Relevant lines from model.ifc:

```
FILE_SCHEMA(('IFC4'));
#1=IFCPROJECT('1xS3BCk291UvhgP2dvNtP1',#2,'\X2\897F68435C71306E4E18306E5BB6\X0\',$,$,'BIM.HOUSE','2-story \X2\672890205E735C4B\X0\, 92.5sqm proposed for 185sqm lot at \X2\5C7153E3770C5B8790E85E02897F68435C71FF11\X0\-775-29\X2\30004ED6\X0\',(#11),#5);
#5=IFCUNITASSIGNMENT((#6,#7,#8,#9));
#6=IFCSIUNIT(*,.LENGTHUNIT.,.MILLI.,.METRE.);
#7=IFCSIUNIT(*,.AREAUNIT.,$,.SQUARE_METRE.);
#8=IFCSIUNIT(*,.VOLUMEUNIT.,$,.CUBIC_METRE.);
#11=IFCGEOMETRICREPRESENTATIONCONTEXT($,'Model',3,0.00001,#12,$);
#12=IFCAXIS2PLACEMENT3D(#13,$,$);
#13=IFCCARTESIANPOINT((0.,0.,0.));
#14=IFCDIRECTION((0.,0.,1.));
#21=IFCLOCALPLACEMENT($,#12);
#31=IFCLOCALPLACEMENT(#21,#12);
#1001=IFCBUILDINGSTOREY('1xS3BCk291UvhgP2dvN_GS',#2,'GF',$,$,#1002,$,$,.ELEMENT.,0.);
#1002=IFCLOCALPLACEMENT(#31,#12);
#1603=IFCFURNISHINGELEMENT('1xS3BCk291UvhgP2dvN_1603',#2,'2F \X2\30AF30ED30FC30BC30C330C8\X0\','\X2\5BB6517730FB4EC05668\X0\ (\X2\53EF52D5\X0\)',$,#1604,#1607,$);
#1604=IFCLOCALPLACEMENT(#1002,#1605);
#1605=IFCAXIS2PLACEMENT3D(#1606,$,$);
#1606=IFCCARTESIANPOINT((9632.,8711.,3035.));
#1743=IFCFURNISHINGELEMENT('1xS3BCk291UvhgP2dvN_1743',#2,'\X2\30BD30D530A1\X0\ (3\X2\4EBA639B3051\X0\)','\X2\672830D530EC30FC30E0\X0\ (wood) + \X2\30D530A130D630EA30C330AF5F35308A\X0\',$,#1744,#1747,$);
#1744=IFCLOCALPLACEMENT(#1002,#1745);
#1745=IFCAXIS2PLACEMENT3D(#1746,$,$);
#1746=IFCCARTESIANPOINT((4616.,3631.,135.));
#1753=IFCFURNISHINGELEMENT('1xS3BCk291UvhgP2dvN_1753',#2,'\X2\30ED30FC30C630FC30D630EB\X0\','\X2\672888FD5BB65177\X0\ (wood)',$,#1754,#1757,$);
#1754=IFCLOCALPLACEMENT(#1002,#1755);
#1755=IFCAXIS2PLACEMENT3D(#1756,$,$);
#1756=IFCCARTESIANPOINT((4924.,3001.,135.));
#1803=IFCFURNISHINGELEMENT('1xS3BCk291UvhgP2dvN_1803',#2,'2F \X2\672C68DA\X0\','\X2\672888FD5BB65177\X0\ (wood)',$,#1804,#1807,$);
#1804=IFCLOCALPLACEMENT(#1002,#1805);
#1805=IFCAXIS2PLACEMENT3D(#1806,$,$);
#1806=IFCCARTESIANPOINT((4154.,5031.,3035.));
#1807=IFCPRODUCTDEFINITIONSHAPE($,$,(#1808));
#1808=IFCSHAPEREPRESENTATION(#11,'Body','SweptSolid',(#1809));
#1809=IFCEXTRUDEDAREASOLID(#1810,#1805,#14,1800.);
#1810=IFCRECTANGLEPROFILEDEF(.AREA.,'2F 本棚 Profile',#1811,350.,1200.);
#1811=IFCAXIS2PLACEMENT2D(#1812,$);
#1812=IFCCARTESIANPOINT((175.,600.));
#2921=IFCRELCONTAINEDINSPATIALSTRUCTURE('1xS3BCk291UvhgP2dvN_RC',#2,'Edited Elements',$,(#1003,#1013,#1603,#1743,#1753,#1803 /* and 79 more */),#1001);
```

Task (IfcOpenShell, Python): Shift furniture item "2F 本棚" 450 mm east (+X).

```python
import ifcopenshell
import ifcopenshell.api.geometry
import ifcopenshell.util.placement

model = ifcopenshell.open("model.ifc")

item = model.by_guid("1xS3BCk291UvhgP2dvN_1803")
matrix = ifcopenshell.util.placement.get_local_placement(item.ObjectPlacement)
matrix[0, 3] += 450.0
ifcopenshell.api.geometry.edit_object_placement(model, product=item, matrix=matrix, is_si=False)

print(ifcopenshell.util.placement.get_local_placement(item.ObjectPlacement).round(3) + 0.0)

model.write("model_updated.ifc")
```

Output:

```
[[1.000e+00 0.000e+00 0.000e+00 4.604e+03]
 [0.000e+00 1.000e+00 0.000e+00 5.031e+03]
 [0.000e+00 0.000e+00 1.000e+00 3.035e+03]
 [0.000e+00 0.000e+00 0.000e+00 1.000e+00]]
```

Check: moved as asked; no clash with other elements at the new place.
